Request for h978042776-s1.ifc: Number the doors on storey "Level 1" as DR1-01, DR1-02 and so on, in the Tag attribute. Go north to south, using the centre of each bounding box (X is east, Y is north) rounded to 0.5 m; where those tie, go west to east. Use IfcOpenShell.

First a look at what the model holds.

```python
import ifcopenshell
import ifcopenshell.util.element
import ifcopenshell.util.placement

model = ifcopenshell.open("h978042776-s1.ifc")
print(model.schema)
storey = next(s for s in model.by_type("IfcBuildingStorey") if s.Name == "Level 1")
doors = [e for e in ifcopenshell.util.element.get_decomposition(storey) if e.is_a("IfcDoor")]
for e in sorted(doors, key=lambda e: e.id()):
    origin = ifcopenshell.util.placement.get_local_placement(e.ObjectPlacement)[:3, 3]
    print(e.id(), e.Tag, e.Name, origin.round(2) + 0.0, sep=" | ")
```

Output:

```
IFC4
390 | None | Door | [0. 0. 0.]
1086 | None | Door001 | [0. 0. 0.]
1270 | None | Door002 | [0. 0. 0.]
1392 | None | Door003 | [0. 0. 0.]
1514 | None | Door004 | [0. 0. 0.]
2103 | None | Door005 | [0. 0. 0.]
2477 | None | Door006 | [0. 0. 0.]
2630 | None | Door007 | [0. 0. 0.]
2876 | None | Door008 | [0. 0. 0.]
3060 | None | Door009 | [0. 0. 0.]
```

```python
import ifcopenshell
import ifcopenshell.geom
import ifcopenshell.util.element
import ifcopenshell.util.shape

model = ifcopenshell.open("h978042776-s1.ifc")
settings = ifcopenshell.geom.settings()
settings.set("use-world-coords", True)


def centre(element):
    shape = ifcopenshell.geom.create_shape(settings, element)
    return ifcopenshell.util.shape.get_bbox_centroid(shape.geometry)


storey = next(s for s in model.by_type("IfcBuildingStorey") if s.Name == "Level 1")
doors = [e for e in ifcopenshell.util.element.get_decomposition(storey) if e.is_a("IfcDoor")]

# Insertion points can sit at a corner or the storey origin, so sort by the geometry (in metres).
centres = {e: centre(e) for e in doors}
doors.sort(key=lambda e: (-round(centres[e][1] / 0.5), centres[e][0]))

for i, e in enumerate(doors, start=1):
    number = f"DR1-{i:02d}"
    e.Tag = number
    print(e.id(), number)

model.write("h978042776-s1_updated.ifc")
```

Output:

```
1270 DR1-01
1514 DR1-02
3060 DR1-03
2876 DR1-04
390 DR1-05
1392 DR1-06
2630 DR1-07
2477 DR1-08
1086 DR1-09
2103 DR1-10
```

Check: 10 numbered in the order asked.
